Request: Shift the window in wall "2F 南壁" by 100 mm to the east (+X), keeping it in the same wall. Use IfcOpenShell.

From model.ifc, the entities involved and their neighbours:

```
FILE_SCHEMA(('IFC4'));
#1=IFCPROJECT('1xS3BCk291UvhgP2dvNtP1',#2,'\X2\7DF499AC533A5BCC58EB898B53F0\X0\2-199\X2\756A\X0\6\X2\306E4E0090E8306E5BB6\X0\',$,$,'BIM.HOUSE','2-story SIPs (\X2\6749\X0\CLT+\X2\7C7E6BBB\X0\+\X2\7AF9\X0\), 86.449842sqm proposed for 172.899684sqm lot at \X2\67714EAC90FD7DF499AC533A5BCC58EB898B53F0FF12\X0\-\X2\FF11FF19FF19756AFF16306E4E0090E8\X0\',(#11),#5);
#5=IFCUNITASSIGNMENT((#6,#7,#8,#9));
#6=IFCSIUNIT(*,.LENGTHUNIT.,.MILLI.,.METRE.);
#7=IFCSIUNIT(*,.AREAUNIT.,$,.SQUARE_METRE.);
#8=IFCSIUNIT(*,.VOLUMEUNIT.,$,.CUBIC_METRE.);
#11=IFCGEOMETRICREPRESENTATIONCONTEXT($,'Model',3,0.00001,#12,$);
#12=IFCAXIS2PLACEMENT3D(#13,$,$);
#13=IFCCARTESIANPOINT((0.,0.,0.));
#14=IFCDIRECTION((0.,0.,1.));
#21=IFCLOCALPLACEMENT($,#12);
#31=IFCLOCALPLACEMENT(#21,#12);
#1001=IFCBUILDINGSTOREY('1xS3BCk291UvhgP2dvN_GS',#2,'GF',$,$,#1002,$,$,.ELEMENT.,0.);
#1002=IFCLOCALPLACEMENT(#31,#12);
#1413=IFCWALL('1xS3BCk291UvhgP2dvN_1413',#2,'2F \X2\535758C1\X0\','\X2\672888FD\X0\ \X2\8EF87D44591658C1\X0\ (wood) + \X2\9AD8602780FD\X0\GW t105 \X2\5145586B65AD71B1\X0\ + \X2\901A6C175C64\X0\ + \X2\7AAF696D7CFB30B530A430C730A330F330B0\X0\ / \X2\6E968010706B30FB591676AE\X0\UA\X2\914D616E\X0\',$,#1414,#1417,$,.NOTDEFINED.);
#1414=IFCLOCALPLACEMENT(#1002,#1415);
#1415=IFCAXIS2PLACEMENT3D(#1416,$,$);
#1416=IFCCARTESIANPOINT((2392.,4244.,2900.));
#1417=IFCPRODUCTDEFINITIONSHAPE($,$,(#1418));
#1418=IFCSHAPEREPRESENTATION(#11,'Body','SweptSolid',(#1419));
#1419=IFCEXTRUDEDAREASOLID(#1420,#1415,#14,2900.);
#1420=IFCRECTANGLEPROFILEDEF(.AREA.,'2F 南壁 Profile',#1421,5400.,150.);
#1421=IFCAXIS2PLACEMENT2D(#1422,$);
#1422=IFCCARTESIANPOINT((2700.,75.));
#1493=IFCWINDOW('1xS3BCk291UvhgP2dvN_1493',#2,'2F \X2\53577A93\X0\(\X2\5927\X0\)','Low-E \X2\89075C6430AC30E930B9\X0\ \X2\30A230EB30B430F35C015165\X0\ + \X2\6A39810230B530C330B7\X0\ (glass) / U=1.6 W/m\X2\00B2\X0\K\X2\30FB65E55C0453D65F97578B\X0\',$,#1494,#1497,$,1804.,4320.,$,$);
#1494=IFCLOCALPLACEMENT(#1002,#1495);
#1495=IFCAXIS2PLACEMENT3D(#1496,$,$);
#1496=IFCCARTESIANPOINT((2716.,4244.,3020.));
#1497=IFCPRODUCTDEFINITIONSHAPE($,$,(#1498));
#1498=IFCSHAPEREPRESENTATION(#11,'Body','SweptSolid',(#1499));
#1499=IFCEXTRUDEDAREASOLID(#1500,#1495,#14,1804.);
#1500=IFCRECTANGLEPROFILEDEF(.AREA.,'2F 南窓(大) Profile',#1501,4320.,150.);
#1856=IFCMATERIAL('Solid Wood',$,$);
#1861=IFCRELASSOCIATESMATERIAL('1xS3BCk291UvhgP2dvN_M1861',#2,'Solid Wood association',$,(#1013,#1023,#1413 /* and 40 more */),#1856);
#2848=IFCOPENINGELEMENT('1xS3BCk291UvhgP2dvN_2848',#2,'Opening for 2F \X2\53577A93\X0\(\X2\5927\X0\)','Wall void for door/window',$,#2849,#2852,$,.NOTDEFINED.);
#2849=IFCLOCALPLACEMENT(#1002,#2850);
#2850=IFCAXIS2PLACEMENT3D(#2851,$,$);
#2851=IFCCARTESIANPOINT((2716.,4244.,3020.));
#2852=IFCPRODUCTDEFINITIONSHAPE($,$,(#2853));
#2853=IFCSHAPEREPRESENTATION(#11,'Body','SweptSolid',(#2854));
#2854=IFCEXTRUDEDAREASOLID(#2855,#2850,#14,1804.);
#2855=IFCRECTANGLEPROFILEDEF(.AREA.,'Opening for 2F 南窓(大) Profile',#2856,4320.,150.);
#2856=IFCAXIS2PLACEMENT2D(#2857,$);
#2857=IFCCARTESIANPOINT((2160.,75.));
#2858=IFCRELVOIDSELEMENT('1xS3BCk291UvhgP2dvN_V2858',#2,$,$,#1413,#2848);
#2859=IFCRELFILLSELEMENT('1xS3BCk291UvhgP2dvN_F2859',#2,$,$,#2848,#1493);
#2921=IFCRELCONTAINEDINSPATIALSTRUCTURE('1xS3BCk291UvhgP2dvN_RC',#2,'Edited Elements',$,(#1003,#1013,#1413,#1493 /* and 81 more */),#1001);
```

```python
import ifcopenshell
import ifcopenshell.api.geometry
import ifcopenshell.util.placement
import ifcopenshell.util.unit

model = ifcopenshell.open("model.ifc")
unit_scale = ifcopenshell.util.unit.calculate_unit_scale(model)

window = model.by_guid("1xS3BCk291UvhgP2dvN_1493")
opening = window.FillsVoids[0].RelatingOpeningElement
wall = opening.VoidsElements[0].RelatingBuildingElement

wall_matrix = ifcopenshell.util.placement.get_local_placement(wall.ObjectPlacement)
shift = wall_matrix[:3, 0] * 0.1 / unit_scale
before = ifcopenshell.util.placement.get_local_placement(window.ObjectPlacement)[:3, 3].copy()

# The window is not placed relative to its opening, so move both.
for product in (opening, window):
    matrix = ifcopenshell.util.placement.get_local_placement(product.ObjectPlacement)
    matrix[:3, 3] += shift
    ifcopenshell.api.geometry.edit_object_placement(model, product=product, matrix=matrix, is_si=False)

after = ifcopenshell.util.placement.get_local_placement(window.ObjectPlacement)[:3, 3]
print("window moved by", (after - before).round(3) + 0.0)

model.write("model_rev.ifc")
```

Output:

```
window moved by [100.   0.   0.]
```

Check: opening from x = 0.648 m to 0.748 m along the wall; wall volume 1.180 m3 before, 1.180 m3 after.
